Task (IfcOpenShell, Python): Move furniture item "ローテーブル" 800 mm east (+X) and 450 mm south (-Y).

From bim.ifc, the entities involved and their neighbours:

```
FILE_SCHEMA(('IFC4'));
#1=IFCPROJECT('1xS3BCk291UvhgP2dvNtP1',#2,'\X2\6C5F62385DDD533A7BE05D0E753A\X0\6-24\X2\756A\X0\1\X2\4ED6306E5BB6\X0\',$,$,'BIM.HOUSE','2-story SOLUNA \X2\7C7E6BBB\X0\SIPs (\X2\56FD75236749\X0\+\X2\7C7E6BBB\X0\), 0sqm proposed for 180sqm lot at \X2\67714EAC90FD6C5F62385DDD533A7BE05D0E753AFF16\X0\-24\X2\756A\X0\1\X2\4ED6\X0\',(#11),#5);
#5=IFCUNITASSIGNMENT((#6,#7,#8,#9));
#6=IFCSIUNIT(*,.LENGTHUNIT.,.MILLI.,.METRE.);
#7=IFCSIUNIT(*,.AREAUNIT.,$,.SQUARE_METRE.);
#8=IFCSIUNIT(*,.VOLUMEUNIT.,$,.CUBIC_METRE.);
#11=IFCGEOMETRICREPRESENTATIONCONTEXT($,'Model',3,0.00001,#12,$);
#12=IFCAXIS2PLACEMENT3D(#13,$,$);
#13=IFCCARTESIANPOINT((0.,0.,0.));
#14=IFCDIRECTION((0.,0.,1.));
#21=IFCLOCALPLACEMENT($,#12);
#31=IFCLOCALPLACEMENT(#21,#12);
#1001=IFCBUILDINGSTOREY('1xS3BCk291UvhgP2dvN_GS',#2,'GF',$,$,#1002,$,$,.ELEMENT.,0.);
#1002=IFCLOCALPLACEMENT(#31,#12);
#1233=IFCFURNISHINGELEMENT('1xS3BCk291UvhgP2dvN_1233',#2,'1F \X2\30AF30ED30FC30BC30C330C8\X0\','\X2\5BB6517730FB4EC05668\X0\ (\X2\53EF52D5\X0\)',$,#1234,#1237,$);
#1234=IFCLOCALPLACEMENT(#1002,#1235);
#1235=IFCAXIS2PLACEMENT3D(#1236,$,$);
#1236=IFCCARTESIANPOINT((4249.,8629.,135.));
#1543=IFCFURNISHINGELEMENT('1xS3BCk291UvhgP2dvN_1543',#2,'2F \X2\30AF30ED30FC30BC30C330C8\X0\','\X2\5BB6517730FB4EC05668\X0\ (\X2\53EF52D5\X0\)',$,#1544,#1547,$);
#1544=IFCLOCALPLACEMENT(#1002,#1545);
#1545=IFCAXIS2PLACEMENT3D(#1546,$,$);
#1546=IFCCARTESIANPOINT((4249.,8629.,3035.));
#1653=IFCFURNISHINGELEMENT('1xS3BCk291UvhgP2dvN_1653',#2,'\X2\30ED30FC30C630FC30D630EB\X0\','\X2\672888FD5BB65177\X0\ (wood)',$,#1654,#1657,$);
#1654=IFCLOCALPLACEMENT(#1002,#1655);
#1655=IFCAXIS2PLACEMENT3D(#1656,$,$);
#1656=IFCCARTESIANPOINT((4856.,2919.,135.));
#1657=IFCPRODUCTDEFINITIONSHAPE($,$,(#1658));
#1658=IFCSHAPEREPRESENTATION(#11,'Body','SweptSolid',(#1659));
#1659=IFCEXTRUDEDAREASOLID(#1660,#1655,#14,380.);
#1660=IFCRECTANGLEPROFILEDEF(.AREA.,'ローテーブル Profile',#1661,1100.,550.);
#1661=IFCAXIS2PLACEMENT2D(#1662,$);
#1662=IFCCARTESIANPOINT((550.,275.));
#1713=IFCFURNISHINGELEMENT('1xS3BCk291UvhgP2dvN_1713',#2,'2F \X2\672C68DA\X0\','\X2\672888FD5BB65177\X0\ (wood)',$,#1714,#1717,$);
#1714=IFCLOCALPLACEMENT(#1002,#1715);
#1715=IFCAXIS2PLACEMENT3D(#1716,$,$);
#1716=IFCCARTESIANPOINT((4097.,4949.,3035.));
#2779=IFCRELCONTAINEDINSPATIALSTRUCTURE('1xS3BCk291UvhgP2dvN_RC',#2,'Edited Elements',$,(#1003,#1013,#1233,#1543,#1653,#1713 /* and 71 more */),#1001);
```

```python
import ifcopenshell
import ifcopenshell.api.geometry
import ifcopenshell.util.placement
import ifcopenshell.util.unit

model = ifcopenshell.open("bim.ifc")
unit_scale = ifcopenshell.util.unit.calculate_unit_scale(model)

item = model.by_id(1653)
matrix = ifcopenshell.util.placement.get_local_placement(item.ObjectPlacement)
matrix[0, 3] += 0.8 / unit_scale
matrix[1, 3] -= 0.45 / unit_scale
ifcopenshell.api.geometry.edit_object_placement(model, product=item, matrix=matrix, is_si=False)

print(ifcopenshell.util.placement.get_local_placement(item.ObjectPlacement).round(3) + 0.0)

model.write("bim_edited.ifc")
```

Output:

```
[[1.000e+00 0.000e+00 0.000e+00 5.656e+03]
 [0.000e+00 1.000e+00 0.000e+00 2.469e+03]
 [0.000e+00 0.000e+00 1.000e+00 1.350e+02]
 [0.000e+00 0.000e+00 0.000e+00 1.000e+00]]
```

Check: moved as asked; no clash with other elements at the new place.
